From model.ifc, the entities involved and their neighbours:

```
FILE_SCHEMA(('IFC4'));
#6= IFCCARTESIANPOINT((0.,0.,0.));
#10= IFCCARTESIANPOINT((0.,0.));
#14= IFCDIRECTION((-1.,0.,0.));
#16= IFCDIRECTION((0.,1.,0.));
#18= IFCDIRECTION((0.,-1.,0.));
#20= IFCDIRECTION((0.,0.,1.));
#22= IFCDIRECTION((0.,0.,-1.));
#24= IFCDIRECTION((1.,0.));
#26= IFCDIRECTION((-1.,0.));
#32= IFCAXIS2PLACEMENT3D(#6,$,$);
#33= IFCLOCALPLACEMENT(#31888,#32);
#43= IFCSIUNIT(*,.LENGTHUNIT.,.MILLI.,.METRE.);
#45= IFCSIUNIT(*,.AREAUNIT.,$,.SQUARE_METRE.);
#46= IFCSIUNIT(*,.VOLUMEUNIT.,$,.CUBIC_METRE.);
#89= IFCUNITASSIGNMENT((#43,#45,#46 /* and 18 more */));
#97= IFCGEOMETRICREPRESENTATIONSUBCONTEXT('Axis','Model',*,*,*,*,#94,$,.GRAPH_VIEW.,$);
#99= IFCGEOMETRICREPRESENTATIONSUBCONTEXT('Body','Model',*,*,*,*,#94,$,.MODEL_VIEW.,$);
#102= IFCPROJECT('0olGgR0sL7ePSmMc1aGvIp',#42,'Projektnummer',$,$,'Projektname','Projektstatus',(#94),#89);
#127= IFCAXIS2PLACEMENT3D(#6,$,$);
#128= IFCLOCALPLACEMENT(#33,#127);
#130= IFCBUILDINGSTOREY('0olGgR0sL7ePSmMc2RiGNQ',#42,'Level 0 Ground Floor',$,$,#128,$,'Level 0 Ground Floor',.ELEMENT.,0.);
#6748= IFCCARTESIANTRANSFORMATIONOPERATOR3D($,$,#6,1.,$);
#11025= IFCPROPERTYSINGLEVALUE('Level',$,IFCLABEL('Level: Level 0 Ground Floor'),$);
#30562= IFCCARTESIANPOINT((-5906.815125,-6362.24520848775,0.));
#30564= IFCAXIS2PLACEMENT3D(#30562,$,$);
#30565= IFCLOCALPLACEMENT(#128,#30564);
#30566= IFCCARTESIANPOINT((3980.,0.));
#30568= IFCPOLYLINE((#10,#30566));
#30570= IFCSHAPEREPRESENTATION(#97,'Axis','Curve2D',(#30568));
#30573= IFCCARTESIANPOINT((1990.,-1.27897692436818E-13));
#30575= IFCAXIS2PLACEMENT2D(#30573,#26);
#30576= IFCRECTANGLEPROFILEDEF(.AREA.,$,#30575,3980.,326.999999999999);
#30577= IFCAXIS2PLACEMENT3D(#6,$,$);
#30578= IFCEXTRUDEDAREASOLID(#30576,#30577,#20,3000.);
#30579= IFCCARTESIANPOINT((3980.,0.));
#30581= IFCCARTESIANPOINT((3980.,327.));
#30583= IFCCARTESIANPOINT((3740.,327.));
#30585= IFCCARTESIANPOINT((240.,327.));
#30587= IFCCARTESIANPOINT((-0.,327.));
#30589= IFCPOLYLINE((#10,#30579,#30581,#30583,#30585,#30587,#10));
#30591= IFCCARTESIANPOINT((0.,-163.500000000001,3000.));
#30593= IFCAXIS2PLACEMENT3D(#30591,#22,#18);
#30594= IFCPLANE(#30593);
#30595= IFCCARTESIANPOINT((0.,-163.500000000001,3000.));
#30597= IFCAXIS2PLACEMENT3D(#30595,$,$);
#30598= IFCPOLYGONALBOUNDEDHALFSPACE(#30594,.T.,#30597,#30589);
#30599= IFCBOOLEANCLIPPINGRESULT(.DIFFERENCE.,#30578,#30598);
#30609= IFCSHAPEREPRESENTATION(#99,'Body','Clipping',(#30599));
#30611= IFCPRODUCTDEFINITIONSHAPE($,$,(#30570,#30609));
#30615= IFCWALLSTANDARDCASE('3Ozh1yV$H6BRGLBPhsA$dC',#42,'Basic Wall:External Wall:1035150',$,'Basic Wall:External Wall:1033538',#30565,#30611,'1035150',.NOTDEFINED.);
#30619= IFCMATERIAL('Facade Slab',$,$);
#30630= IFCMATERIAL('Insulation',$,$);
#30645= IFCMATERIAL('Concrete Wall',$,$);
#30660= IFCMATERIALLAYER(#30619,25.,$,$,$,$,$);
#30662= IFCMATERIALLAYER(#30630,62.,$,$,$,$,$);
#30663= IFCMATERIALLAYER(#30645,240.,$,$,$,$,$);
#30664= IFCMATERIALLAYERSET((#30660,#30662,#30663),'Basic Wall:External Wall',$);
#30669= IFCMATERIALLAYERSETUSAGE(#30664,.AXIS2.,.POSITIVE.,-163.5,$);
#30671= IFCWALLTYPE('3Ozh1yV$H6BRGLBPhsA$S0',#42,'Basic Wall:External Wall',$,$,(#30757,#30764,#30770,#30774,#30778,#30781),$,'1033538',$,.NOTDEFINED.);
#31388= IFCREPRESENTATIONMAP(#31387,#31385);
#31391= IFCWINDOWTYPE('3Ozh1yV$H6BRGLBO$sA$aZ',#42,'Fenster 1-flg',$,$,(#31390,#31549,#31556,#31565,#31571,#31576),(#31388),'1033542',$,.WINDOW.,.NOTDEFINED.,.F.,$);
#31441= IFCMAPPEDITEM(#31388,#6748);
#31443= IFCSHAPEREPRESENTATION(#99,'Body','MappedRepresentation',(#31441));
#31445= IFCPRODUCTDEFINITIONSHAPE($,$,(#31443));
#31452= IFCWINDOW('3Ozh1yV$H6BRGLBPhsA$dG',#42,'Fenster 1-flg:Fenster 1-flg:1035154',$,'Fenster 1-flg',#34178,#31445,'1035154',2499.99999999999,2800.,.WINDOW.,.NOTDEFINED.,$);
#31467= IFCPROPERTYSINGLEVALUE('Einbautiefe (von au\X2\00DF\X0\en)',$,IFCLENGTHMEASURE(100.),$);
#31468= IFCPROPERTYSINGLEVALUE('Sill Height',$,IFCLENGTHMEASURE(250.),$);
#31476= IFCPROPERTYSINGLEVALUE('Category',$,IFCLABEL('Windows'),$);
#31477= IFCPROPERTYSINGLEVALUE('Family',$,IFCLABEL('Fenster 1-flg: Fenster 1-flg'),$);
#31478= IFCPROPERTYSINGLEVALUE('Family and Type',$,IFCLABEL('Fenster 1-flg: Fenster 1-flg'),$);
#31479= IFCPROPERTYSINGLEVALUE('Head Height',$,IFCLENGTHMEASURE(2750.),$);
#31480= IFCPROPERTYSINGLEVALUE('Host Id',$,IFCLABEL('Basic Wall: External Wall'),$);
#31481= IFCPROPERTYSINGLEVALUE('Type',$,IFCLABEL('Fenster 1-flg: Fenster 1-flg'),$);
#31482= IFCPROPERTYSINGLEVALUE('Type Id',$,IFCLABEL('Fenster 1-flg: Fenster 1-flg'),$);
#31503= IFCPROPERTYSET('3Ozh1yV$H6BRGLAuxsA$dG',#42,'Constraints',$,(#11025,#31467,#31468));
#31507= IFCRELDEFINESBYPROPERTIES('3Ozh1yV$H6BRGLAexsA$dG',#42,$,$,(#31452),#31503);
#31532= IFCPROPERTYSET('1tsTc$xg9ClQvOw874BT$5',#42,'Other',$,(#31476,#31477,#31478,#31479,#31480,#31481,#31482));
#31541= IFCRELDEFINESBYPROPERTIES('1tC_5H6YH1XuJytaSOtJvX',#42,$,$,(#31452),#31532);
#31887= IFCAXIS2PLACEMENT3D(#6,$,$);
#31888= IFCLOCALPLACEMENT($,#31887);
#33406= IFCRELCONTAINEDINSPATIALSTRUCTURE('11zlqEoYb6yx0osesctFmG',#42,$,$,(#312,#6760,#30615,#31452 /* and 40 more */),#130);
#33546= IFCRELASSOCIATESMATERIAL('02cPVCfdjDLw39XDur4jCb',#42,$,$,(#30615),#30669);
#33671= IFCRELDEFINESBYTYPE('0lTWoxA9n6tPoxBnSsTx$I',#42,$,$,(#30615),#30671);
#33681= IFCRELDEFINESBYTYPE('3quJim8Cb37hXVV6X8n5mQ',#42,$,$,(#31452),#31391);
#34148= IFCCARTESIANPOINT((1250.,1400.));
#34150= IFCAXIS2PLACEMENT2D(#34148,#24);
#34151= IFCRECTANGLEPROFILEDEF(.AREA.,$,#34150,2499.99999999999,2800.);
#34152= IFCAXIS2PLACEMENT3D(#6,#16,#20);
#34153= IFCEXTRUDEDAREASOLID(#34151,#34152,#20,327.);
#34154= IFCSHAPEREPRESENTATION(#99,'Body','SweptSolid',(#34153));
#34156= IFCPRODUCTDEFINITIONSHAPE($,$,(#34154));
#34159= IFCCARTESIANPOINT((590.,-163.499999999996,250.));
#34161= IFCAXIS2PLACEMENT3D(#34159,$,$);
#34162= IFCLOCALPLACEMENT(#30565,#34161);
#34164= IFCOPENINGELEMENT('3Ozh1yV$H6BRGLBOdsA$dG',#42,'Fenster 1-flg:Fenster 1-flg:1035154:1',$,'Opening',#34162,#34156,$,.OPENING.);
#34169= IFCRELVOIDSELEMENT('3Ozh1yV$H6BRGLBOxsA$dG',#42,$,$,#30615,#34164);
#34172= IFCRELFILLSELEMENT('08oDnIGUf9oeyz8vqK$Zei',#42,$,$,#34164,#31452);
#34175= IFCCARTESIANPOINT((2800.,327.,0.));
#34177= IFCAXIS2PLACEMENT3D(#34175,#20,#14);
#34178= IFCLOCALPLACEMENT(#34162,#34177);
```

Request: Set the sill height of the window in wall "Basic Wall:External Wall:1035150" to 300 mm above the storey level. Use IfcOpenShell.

```python
import numpy as np
import ifcopenshell
import ifcopenshell.api.geometry
import ifcopenshell.api.pset
import ifcopenshell.geom
import ifcopenshell.util.element
import ifcopenshell.util.placement
import ifcopenshell.util.shape
import ifcopenshell.util.unit

model = ifcopenshell.open("model.ifc")
unit_scale = ifcopenshell.util.unit.calculate_unit_scale(model)

window = model.by_id(31452)
opening = window.FillsVoids[0].RelatingOpeningElement
storey = ifcopenshell.util.element.get_container(window, ifc_class="IfcBuildingStorey")
level = ifcopenshell.util.placement.get_local_placement(storey.ObjectPlacement)[2, 3]

# The opening's origin need not be at the sill, so measure its lowest point.
shape = ifcopenshell.geom.create_shape(ifcopenshell.geom.settings(), opening)
bottom = ifcopenshell.util.shape.get_shape_bottom_elevation(shape, shape.geometry) / unit_scale
dz = level + 300.0 - bottom

shift = np.array([0.0, 0.0, dz])
# The window is placed relative to its opening, so it follows when the opening moves.
matrix = ifcopenshell.util.placement.get_local_placement(opening.ObjectPlacement)
matrix[:3, 3] += shift
ifcopenshell.api.geometry.edit_object_placement(
    model, product=opening, matrix=matrix, is_si=False, should_transform_children=True
)

# Keep the stored heights in step.
pset = model.by_id(ifcopenshell.util.element.get_pset(window, "Constraints", should_inherit=False)["id"])
ifcopenshell.api.pset.edit_pset(model, pset=pset, properties={
    "Sill Height": model.create_entity("IfcLengthMeasure", ifcopenshell.util.element.get_pset(window, "Constraints", "Sill Height") + dz),
})
pset = model.by_id(ifcopenshell.util.element.get_pset(window, "Other", should_inherit=False)["id"])
ifcopenshell.api.pset.edit_pset(model, pset=pset, properties={
    "Head Height": model.create_entity("IfcLengthMeasure", ifcopenshell.util.element.get_pset(window, "Other", "Head Height") + dz),
})

print(f"moved by {dz * unit_scale:+.3f} m")

model.write("model_rev.ifc")
```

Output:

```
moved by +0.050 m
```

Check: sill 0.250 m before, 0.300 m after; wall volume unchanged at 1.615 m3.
